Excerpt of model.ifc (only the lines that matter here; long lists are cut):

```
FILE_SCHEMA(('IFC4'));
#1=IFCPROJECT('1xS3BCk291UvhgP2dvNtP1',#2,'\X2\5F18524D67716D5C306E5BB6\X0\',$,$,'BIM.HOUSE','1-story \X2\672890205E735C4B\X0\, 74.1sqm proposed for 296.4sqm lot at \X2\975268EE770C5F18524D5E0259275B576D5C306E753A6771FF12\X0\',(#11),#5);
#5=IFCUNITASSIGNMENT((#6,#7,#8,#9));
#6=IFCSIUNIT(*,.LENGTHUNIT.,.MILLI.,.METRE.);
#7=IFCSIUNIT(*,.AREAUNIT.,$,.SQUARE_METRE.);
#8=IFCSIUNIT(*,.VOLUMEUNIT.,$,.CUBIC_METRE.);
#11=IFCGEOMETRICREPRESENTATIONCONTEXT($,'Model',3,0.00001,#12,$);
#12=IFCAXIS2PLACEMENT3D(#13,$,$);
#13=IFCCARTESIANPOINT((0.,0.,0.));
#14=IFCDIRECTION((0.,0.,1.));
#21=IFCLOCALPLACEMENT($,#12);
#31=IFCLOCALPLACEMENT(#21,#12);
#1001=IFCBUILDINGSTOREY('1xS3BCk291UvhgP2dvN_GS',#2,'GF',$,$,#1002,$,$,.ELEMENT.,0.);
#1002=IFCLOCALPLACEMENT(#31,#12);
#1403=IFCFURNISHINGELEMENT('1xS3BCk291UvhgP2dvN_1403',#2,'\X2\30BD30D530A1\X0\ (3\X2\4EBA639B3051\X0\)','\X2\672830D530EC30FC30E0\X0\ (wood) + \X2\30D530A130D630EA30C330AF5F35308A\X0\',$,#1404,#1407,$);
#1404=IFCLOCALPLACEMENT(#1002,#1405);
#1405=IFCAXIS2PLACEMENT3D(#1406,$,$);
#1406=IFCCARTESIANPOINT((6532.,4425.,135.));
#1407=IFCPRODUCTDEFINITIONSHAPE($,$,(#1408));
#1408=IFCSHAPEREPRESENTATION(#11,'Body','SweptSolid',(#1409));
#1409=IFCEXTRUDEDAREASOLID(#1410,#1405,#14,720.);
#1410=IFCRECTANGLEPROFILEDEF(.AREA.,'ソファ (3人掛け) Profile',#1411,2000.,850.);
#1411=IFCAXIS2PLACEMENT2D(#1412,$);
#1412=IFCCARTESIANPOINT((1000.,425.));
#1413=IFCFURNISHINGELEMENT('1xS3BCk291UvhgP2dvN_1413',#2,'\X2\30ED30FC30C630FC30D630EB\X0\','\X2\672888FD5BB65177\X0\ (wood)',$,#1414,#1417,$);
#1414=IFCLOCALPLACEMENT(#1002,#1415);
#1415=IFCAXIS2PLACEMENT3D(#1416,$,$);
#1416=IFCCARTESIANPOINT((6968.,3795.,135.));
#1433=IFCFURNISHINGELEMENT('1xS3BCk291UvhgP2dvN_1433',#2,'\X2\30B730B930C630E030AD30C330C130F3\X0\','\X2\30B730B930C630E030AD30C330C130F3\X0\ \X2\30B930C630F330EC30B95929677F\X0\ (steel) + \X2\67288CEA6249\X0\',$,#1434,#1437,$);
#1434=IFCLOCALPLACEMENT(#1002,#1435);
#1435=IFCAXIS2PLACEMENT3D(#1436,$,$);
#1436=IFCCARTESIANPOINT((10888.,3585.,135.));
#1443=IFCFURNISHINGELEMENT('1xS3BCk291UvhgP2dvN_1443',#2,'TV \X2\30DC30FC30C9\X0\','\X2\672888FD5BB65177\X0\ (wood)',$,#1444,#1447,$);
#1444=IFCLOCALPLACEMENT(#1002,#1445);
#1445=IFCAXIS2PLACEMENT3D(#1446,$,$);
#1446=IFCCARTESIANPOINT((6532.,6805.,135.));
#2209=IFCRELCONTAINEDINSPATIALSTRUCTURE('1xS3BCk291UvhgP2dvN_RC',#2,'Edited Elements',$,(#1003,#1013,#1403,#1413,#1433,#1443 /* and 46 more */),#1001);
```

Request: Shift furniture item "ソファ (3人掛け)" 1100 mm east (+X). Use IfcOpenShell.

```python
import ifcopenshell
import ifcopenshell.api.geometry
import ifcopenshell.util.placement
import ifcopenshell.util.unit

model = ifcopenshell.open("model.ifc")
unit_scale = ifcopenshell.util.unit.calculate_unit_scale(model)

item = model.by_id(1403)
matrix = ifcopenshell.util.placement.get_local_placement(item.ObjectPlacement)
matrix[0, 3] += 1.1 / unit_scale
ifcopenshell.api.geometry.edit_object_placement(model, product=item, matrix=matrix, is_si=False)

print(ifcopenshell.util.placement.get_local_placement(item.ObjectPlacement).round(3) + 0.0)

model.write("model_rev.ifc")
```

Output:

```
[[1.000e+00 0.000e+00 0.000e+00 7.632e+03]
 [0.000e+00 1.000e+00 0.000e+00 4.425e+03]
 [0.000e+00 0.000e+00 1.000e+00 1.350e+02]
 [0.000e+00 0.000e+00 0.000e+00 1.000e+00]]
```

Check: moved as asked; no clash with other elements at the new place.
